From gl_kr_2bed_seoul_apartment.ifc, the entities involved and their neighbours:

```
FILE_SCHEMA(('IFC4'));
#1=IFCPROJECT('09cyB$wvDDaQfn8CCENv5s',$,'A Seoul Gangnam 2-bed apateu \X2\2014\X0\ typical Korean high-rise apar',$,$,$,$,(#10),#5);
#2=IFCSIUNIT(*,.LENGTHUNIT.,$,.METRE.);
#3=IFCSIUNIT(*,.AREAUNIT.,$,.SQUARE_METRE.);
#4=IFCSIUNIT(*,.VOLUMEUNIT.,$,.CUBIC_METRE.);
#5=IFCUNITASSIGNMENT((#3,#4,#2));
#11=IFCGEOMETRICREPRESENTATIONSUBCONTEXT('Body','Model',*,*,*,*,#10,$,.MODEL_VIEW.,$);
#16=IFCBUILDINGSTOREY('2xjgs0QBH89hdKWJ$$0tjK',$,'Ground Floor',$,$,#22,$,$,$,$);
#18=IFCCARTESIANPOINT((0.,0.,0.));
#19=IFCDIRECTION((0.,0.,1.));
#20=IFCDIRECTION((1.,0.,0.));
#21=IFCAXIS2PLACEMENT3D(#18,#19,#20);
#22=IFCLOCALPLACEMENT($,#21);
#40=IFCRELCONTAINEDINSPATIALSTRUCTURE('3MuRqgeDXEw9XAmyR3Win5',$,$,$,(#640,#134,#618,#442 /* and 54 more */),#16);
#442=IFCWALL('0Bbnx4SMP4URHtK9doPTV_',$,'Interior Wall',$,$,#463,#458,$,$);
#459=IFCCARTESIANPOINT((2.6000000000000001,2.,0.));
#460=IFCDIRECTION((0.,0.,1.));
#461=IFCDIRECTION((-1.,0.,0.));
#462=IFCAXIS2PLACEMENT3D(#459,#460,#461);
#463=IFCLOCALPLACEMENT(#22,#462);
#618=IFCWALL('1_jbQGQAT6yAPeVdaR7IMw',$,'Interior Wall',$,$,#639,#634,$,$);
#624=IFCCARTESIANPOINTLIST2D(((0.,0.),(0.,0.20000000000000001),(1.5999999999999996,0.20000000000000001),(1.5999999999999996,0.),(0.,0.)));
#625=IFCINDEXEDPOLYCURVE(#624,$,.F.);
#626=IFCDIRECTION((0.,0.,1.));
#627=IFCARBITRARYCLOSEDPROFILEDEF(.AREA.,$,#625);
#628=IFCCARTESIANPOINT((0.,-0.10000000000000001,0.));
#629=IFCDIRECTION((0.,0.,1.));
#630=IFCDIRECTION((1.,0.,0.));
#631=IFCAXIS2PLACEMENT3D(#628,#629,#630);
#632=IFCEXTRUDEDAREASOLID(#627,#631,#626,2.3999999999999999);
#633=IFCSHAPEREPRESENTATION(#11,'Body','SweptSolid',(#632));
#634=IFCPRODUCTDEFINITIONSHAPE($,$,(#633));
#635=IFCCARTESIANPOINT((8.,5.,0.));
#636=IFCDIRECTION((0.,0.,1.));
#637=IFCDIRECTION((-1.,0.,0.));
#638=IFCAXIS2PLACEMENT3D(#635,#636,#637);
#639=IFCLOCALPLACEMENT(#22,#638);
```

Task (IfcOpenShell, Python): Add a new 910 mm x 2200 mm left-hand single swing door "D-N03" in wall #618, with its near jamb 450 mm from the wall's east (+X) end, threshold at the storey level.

```python
import numpy as np
import ifcopenshell
import ifcopenshell.api.feature
import ifcopenshell.api.geometry
import ifcopenshell.api.root
import ifcopenshell.api.spatial
import ifcopenshell.geom
import ifcopenshell.util.element
import ifcopenshell.util.placement
import ifcopenshell.util.representation
import ifcopenshell.util.shape
import ifcopenshell.util.unit

model = ifcopenshell.open("gl_kr_2bed_seoul_apartment.ifc")
unit_scale = ifcopenshell.util.unit.calculate_unit_scale(model)
settings = ifcopenshell.geom.settings()


def volume(element):
    """Net volume in cubic metres, openings subtracted."""
    shape = ifcopenshell.geom.create_shape(settings, element)
    return ifcopenshell.util.shape.get_volume(shape.geometry)


wall = model.by_guid("1_jbQGQAT6yAPeVdaR7IMw")
storey = ifcopenshell.util.element.get_container(wall, ifc_class="IfcBuildingStorey")
context = ifcopenshell.util.representation.get_context(model, "Model", "Body", "MODEL_VIEW")
before = volume(wall)

width, height, from_end, sill = 0.91, 2.2, 0.45, 0.0  # metres

# The wall runs along its own X axis, and the end named is its -X end.
wall_shape = ifcopenshell.geom.create_shape(settings, wall)
x, y, z = ifcopenshell.util.shape.get_vertices(wall_shape.geometry).T
start = x.min() + from_end
face, thickness = float(y.min()), float(y.max() - y.min())
wall_matrix = ifcopenshell.util.placement.get_local_placement(wall.ObjectPlacement)
level = ifcopenshell.util.placement.get_local_placement(storey.ObjectPlacement)[2, 3]


def in_wall(x, y):
    """Placement at x, y metres in the wall's axes, at sill height."""
    matrix = wall_matrix.copy()
    matrix[:, 3] = wall_matrix @ np.array([x / unit_scale, y / unit_scale, 0.0, 1.0])
    matrix[2, 3] = level + sill / unit_scale
    return matrix


# Opening: a box that overshoots both wall faces by 50 mm.
opening = ifcopenshell.api.root.create_entity(model, ifc_class="IfcOpeningElement", predefined_type="OPENING")
box = ifcopenshell.api.geometry.add_wall_representation(
    model, context=context, length=width, height=height, thickness=thickness + 0.1
)
ifcopenshell.api.geometry.assign_representation(model, product=opening, representation=box)
ifcopenshell.api.geometry.edit_object_placement(model, product=opening, matrix=in_wall(start, face - 0.05), is_si=False)
ifcopenshell.api.feature.add_feature(model, feature=opening, element=wall)

door = ifcopenshell.api.root.create_entity(model, ifc_class="IfcDoor", name="D-N03", predefined_type="DOOR")
door.OverallWidth, door.OverallHeight = width / unit_scale, height / unit_scale
door.OperationType = "SINGLE_SWING_LEFT"
body = ifcopenshell.api.geometry.add_door_representation(
    model,
    context=context,
    overall_width=door.OverallWidth,
    overall_height=door.OverallHeight,
    operation_type="SINGLE_SWING_LEFT",
    lining_properties={"LiningDepth": thickness / unit_scale, "ThresholdDepth": thickness / unit_scale},
)
ifcopenshell.api.geometry.assign_representation(model, product=door, representation=body)
ifcopenshell.api.spatial.assign_container(model, products=[door], relating_structure=storey)
ifcopenshell.api.feature.add_filling(model, opening=opening, element=door)

# The lining spans the wall, so the door starts at the wall face.
ifcopenshell.api.geometry.edit_object_placement(model, product=door, matrix=in_wall(start, face), is_si=False)

after = volume(wall)

print(f"wall volume {before:.3f} -> {after:.3f} m3")

model.write("gl_kr_2bed_seoul_apartment_edited.ifc")
```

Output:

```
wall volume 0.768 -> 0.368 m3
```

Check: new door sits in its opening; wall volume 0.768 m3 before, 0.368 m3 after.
